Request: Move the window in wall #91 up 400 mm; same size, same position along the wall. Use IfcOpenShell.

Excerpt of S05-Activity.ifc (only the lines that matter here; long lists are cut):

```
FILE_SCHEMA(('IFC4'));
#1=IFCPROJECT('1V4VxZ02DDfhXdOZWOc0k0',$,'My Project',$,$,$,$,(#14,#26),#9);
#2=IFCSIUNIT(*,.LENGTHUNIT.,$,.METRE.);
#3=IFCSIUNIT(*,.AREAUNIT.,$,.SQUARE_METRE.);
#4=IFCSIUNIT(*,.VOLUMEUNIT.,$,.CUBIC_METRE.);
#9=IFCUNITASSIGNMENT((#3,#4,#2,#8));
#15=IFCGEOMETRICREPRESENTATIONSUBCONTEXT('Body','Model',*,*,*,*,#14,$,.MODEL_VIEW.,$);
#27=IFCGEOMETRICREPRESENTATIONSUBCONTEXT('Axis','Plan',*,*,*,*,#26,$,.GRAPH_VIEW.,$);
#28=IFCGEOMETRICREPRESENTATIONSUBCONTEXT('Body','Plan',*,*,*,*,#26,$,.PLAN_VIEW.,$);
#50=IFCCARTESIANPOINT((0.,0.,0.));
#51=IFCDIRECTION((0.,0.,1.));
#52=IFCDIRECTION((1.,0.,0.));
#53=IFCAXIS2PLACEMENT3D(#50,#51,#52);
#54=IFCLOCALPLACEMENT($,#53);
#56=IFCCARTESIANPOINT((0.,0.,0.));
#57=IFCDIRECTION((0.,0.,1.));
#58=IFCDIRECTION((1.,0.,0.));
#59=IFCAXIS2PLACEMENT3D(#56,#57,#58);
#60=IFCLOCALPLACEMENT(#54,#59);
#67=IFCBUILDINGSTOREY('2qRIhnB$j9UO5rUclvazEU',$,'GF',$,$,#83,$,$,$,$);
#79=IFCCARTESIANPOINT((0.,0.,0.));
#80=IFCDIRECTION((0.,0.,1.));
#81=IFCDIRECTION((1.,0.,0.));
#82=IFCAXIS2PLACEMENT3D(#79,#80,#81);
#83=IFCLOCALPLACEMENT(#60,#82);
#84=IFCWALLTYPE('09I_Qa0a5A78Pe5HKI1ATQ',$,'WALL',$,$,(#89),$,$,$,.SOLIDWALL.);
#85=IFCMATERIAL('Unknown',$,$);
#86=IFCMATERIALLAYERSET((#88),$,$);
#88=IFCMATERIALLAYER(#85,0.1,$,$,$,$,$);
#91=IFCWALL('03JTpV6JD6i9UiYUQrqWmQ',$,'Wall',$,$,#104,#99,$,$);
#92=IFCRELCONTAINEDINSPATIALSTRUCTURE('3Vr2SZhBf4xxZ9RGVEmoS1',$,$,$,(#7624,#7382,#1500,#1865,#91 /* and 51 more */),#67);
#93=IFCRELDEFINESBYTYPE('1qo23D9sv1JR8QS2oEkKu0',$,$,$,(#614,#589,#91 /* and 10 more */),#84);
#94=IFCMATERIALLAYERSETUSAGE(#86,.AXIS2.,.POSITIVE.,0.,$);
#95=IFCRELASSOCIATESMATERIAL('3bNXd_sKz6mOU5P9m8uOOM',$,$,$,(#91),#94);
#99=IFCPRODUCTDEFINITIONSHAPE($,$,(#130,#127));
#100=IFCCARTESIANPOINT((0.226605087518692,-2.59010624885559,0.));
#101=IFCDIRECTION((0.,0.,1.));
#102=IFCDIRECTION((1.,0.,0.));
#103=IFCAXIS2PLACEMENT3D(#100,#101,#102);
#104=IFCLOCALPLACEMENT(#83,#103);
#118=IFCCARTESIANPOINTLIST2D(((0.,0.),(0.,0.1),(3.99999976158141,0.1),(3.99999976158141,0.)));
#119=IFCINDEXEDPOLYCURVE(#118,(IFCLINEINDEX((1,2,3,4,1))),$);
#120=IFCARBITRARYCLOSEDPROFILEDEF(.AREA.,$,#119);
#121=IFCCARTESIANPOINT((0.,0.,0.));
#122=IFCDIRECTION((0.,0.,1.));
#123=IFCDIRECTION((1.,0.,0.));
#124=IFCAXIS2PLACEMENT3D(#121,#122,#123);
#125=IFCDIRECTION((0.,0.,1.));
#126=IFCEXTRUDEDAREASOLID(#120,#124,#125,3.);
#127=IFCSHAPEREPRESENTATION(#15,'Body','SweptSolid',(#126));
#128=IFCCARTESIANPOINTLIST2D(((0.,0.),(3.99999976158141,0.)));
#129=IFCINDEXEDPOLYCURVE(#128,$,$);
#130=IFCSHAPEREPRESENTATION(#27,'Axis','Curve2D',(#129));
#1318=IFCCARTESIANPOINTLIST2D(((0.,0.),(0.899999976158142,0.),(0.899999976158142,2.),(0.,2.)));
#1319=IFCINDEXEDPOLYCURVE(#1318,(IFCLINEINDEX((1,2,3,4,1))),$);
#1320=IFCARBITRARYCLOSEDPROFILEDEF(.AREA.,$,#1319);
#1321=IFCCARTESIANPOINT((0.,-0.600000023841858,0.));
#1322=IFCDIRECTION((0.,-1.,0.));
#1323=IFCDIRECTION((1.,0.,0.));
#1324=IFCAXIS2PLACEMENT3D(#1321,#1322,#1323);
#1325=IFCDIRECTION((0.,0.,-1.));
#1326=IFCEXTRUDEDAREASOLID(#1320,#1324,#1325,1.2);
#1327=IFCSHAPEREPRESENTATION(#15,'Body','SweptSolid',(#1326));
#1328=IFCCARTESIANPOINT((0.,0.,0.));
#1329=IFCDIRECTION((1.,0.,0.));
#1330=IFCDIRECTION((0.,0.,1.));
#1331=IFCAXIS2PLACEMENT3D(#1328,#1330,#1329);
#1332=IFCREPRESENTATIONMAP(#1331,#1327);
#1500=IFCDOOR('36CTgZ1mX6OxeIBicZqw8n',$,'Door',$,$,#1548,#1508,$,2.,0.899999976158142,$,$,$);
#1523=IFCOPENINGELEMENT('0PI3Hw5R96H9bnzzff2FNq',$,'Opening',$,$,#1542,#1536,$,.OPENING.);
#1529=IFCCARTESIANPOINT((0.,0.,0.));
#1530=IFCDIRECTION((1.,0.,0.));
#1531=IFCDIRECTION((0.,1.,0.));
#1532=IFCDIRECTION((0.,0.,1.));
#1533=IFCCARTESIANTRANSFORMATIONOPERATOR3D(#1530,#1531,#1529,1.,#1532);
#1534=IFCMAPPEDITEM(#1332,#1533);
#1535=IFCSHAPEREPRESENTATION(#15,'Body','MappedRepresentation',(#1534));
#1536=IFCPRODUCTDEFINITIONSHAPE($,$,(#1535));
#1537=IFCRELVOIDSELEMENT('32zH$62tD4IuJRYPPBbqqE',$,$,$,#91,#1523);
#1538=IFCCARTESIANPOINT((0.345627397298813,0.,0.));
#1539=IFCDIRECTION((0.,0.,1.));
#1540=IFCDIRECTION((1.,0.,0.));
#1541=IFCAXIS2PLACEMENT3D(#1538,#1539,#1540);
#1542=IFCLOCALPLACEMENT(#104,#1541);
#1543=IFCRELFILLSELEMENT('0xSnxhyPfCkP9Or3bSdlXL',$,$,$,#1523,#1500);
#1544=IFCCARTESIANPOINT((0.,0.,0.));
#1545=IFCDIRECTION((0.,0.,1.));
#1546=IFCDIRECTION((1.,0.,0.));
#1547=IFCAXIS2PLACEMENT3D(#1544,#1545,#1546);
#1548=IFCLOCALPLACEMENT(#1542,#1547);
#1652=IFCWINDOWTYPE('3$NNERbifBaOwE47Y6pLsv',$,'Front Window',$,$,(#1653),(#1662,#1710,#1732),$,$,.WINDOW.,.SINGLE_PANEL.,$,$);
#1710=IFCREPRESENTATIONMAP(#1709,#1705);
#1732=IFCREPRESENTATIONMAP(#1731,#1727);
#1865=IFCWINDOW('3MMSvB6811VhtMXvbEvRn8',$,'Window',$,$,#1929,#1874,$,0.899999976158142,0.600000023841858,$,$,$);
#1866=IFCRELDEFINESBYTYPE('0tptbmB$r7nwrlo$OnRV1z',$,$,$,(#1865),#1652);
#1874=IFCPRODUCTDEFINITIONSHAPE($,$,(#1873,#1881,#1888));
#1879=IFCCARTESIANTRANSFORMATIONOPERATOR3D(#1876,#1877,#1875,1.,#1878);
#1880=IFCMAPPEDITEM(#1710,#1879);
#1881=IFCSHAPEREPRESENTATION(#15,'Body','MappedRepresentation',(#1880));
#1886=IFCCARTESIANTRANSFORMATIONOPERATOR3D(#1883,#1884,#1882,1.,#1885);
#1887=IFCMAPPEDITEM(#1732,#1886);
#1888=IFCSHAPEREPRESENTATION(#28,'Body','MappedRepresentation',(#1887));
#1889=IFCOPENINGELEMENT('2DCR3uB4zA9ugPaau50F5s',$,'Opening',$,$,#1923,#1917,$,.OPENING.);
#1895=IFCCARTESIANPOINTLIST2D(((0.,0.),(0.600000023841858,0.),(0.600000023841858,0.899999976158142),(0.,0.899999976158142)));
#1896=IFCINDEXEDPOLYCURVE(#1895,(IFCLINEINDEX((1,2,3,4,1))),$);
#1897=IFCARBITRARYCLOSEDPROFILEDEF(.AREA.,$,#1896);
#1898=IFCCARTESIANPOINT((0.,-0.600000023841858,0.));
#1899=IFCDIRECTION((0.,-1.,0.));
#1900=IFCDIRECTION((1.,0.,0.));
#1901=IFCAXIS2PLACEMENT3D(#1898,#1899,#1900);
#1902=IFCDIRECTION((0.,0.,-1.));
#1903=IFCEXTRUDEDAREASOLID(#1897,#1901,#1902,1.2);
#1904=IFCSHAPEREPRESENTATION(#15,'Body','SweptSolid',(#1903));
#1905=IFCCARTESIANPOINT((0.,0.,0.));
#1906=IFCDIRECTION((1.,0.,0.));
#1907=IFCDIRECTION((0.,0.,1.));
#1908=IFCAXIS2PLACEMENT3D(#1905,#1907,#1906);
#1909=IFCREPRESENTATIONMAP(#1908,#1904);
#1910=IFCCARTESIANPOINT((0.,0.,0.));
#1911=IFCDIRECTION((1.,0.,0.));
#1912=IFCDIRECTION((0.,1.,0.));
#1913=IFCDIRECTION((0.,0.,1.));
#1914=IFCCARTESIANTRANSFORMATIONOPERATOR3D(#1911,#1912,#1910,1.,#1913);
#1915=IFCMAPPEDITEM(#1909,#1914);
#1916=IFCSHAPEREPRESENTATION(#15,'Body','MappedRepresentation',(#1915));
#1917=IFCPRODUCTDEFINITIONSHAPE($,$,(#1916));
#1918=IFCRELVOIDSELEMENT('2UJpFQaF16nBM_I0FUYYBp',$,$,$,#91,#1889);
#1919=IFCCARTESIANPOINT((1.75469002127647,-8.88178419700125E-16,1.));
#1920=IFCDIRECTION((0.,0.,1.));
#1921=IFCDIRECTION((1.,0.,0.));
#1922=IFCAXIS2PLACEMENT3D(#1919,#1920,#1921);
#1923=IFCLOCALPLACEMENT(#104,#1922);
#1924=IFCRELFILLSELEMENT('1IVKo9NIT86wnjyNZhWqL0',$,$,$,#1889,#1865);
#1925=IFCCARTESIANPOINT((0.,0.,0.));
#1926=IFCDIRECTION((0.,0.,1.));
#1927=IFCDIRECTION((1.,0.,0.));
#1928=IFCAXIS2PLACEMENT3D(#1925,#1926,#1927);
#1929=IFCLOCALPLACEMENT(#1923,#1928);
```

```python
import numpy as np
import ifcopenshell
import ifcopenshell.api.geometry
import ifcopenshell.util.placement
import ifcopenshell.util.unit

model = ifcopenshell.open("S05-Activity.ifc")
unit_scale = ifcopenshell.util.unit.calculate_unit_scale(model)

window = model.by_guid("3MMSvB6811VhtMXvbEvRn8")
opening = window.FillsVoids[0].RelatingOpeningElement
dz = 0.4

shift = np.array([0.0, 0.0, dz])
# The window is placed relative to its opening, so it follows when the opening moves.
matrix = ifcopenshell.util.placement.get_local_placement(opening.ObjectPlacement)
matrix[:3, 3] += shift
ifcopenshell.api.geometry.edit_object_placement(
    model, product=opening, matrix=matrix, is_si=False, should_transform_children=True
)

print(f"moved by {dz * unit_scale:+.3f} m")

model.write("S05-Activity_v2.ifc")
```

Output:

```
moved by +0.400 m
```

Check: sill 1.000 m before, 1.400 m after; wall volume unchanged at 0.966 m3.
